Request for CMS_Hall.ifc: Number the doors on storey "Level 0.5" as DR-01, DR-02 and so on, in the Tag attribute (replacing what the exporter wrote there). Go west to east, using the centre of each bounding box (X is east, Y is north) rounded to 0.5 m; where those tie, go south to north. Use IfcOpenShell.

First a look at what the model holds.

```python
import ifcopenshell
import ifcopenshell.util.element
import ifcopenshell.util.placement

model = ifcopenshell.open("CMS_Hall.ifc")
print(model.schema)
storey = next(s for s in model.by_type("IfcBuildingStorey") if s.Name == "Level 0.5")
doors = [e for e in ifcopenshell.util.element.get_decomposition(storey) if e.is_a("IfcDoor")]
for e in sorted(doors, key=lambda e: e.id()):
    origin = ifcopenshell.util.placement.get_local_placement(e.ObjectPlacement)[:3, 3]
    print(e.id(), e.Tag, e.Name, origin.round(2) + 0.0, sep=" | ")
```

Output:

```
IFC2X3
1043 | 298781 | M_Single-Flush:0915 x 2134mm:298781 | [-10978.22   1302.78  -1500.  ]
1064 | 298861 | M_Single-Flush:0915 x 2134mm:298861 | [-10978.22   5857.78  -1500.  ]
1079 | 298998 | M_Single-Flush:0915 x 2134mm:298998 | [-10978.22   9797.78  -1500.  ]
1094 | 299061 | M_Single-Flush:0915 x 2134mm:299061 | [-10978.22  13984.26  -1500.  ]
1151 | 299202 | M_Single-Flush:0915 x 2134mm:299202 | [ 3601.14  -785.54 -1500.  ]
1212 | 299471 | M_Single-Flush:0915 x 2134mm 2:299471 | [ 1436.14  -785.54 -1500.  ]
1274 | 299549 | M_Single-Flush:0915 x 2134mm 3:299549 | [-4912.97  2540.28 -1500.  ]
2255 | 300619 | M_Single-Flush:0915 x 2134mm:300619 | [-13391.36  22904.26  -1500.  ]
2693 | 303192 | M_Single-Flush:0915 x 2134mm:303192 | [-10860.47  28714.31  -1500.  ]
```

```python
import ifcopenshell
import ifcopenshell.geom
import ifcopenshell.util.element
import ifcopenshell.util.shape

model = ifcopenshell.open("CMS_Hall.ifc")
settings = ifcopenshell.geom.settings()
settings.set("use-world-coords", True)


def centre(element):
    shape = ifcopenshell.geom.create_shape(settings, element)
    return ifcopenshell.util.shape.get_bbox_centroid(shape.geometry)


storey = next(s for s in model.by_type("IfcBuildingStorey") if s.Name == "Level 0.5")
doors = [e for e in ifcopenshell.util.element.get_decomposition(storey) if e.is_a("IfcDoor")]

# Insertion points can sit at a corner or the storey origin, so sort by the geometry (in metres).
centres = {e: centre(e) for e in doors}
doors.sort(key=lambda e: (round(centres[e][0] / 0.5), centres[e][1]))

for i, e in enumerate(doors, start=1):
    number = f"DR-{i:02d}"
    e.Tag = number
    print(e.id(), number)

model.write("CMS_Hall_edited.ifc")
```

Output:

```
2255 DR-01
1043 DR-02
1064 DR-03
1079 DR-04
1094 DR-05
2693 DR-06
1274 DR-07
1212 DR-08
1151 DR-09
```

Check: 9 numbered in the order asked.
